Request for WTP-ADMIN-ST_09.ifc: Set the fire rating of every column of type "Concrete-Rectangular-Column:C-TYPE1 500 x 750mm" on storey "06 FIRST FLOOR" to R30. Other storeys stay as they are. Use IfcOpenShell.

First a look at what the model holds.

```python
import ifcopenshell
import ifcopenshell.util.element

model = ifcopenshell.open("WTP-ADMIN-ST_09.ifc")
print(model.schema)
storey = next(s for s in model.by_type("IfcBuildingStorey") if s.Name == "06 FIRST FLOOR")
columns = [e for e in ifcopenshell.util.element.get_decomposition(storey) if e.is_a("IfcColumn")]
seen = {}
for e in columns:
    element_type = ifcopenshell.util.element.get_type(e)
    key = (element_type.Name if element_type != e and element_type else None, ifcopenshell.util.element.get_pset(e, "Pset_ColumnCommon", "FireRating"))
    seen[key] = seen.get(key, 0) + 1
for (name, value), count in sorted(seen.items(), key=str):
    print(count, "x", name, "|", value)
```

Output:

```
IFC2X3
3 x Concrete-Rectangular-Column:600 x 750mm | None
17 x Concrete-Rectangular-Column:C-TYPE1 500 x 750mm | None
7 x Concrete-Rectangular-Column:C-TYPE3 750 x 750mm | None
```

```python
import ifcopenshell
import ifcopenshell.api.pset
import ifcopenshell.util.element

model = ifcopenshell.open("WTP-ADMIN-ST_09.ifc")

storey = next(s for s in model.by_type("IfcBuildingStorey") if s.Name == "06 FIRST FLOOR")
columns = [e for e in ifcopenshell.util.element.get_decomposition(storey) if e.is_a("IfcColumn")]

count = 0
for e in columns:
    element_type = ifcopenshell.util.element.get_type(e)
    if element_type in (None, e) or element_type.Name != "Concrete-Rectangular-Column:C-TYPE1 500 x 750mm":
        continue
    # add_pset returns the element's existing set when there is one.
    pset = ifcopenshell.api.pset.add_pset(model, product=e, name="Pset_ColumnCommon")
    ifcopenshell.api.pset.edit_pset(model, pset=pset, properties={"FireRating": "R30"})
    count += 1

print(count, "columns updated")

model.write("WTP-ADMIN-ST_09_v2.ifc")
```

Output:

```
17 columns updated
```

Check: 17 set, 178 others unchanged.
